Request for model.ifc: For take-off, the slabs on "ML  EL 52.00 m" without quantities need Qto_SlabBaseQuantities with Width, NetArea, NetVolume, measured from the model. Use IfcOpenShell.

First a look at what the model holds.

```python
import ifcopenshell
import ifcopenshell.util.element
import ifcopenshell.util.unit

model = ifcopenshell.open("model.ifc")
print(model.schema)
for unit_type in ("LENGTHUNIT", "AREAUNIT", "VOLUMEUNIT"):
    print(unit_type, ifcopenshell.util.unit.calculate_unit_scale(model, unit_type))
storey = next(s for s in model.by_type("IfcBuildingStorey") if s.Name == "ML  EL 52.00 m")
slabs = [e for e in ifcopenshell.util.element.get_decomposition(storey) if e.is_a("IfcSlab")]
for e in sorted(slabs, key=lambda e: e.id()):
    print(e.id(), e.is_a(), e.Name, list(ifcopenshell.util.element.get_psets(e, qtos_only=True)), sep=" | ")
```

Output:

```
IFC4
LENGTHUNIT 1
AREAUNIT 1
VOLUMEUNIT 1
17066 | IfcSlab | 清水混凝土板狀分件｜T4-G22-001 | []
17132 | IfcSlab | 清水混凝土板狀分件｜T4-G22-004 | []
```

```python
import ifcopenshell
import ifcopenshell.api.pset
import ifcopenshell.geom
import ifcopenshell.util.element
import ifcopenshell.util.shape
import ifcopenshell.util.unit

model = ifcopenshell.open("model.ifc")
unit_scale = ifcopenshell.util.unit.calculate_unit_scale(model)
area_scale = ifcopenshell.util.unit.calculate_unit_scale(model, "AREAUNIT")
volume_scale = ifcopenshell.util.unit.calculate_unit_scale(model, "VOLUMEUNIT")
settings = ifcopenshell.geom.settings()

storey = next(s for s in model.by_type("IfcBuildingStorey") if s.Name == "ML  EL 52.00 m")
slabs = [e for e in ifcopenshell.util.element.get_decomposition(storey) if e.is_a("IfcSlab")]

for e in sorted(slabs, key=lambda e: e.id()):
    if ifcopenshell.util.element.get_psets(e, qtos_only=True, should_inherit=False):
        continue
    # Geometry comes back in metres, in the element's own axes.
    shape = ifcopenshell.geom.create_shape(settings, e)
    values = {
        "Width": ifcopenshell.util.shape.get_z(shape.geometry) / unit_scale,
        "NetArea": ifcopenshell.util.shape.get_footprint_area(shape.geometry) / area_scale,
        "NetVolume": ifcopenshell.util.shape.get_volume(shape.geometry) / volume_scale,
    }
    qto = ifcopenshell.api.pset.add_qto(model, product=e, name="Qto_SlabBaseQuantities")
    ifcopenshell.api.pset.edit_qto(model, qto=qto, properties=values)
    print(e.id(), {k: round(v, 3) for k, v in values.items()})

model.write("model_edited.ifc")
```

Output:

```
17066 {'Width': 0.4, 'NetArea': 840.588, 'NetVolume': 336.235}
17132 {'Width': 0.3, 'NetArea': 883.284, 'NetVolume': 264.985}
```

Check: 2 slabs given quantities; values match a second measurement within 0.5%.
